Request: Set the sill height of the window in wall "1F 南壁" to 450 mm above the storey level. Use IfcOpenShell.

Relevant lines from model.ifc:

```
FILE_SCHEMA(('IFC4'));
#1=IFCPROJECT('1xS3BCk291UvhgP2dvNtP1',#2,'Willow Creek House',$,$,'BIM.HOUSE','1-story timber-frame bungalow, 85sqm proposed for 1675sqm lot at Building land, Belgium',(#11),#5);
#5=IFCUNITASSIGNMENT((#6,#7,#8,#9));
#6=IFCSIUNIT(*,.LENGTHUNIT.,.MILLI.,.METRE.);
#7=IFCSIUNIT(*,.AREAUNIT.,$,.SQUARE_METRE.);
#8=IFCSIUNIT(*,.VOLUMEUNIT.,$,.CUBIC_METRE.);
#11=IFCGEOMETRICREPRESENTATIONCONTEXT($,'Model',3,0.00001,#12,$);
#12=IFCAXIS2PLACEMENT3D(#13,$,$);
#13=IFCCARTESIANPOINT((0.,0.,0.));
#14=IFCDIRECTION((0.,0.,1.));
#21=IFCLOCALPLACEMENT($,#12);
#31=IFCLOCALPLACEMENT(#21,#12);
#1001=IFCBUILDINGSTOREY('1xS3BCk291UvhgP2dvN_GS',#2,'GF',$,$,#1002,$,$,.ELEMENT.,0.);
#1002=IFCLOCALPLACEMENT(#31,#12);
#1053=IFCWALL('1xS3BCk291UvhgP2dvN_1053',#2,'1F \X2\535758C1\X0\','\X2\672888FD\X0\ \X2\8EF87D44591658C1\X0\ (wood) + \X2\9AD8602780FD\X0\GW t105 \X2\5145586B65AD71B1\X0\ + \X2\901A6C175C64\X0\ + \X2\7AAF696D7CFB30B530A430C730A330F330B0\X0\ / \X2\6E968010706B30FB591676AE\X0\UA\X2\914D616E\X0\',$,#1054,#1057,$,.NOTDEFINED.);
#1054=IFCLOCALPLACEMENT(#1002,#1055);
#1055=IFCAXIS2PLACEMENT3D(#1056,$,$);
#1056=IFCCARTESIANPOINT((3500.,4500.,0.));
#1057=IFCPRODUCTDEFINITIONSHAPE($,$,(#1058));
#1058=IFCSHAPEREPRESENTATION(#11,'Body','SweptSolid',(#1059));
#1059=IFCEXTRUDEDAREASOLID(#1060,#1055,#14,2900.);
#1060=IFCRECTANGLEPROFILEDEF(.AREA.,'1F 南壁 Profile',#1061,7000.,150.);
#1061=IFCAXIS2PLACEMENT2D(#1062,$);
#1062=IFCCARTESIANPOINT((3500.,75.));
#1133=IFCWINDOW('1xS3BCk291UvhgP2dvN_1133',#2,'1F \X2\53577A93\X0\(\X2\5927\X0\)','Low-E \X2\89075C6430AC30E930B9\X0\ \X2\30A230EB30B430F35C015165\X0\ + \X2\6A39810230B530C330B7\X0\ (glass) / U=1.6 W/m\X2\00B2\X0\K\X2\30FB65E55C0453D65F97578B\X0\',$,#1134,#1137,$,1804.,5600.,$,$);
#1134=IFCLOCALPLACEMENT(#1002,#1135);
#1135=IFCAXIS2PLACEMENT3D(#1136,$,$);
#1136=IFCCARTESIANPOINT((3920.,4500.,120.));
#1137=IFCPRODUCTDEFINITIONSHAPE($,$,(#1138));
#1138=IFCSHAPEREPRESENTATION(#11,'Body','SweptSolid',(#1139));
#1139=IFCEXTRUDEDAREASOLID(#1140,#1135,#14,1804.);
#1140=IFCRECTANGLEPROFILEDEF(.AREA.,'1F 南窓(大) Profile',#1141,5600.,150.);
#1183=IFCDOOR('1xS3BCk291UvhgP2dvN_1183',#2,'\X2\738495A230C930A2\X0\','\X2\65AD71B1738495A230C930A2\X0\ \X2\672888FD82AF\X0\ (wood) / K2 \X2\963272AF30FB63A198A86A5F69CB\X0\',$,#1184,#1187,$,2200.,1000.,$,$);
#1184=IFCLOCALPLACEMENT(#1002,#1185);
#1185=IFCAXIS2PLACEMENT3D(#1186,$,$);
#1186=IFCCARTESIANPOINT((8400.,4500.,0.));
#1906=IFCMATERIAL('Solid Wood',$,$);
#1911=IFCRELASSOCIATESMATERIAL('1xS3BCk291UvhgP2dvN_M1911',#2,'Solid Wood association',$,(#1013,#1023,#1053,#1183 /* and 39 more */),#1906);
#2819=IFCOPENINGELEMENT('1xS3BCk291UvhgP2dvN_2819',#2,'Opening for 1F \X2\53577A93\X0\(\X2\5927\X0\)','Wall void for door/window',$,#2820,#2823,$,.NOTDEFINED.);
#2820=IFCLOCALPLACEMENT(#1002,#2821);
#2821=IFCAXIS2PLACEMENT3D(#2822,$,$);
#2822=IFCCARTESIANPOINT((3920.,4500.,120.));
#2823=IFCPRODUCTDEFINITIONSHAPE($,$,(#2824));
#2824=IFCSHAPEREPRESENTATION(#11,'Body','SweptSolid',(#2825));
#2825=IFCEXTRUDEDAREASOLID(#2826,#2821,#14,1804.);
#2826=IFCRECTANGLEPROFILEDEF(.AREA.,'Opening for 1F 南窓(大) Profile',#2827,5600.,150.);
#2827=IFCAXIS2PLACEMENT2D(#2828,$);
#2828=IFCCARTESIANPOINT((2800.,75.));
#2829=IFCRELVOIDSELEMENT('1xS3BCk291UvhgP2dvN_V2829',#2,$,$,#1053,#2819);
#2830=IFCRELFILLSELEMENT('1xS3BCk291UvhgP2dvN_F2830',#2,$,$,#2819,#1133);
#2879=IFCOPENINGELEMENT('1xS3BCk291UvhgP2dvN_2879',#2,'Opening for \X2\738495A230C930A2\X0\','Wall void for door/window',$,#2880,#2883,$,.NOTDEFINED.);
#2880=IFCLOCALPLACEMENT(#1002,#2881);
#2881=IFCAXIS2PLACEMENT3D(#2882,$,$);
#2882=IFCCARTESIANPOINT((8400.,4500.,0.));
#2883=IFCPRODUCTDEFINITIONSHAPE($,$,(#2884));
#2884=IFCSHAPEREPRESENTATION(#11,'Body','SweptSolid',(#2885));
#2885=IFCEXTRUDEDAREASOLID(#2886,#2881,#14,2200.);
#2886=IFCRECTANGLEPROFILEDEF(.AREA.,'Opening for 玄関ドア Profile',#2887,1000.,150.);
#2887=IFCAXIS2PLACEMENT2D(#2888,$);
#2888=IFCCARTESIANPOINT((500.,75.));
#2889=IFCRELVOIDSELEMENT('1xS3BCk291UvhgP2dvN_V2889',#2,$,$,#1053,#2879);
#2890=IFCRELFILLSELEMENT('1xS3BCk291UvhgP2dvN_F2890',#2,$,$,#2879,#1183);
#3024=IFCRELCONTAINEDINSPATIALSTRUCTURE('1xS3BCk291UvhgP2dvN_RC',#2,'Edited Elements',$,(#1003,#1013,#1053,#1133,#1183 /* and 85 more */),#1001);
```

```python
import numpy as np
import ifcopenshell
import ifcopenshell.api.geometry
import ifcopenshell.geom
import ifcopenshell.util.element
import ifcopenshell.util.placement
import ifcopenshell.util.shape
import ifcopenshell.util.unit

model = ifcopenshell.open("model.ifc")
unit_scale = ifcopenshell.util.unit.calculate_unit_scale(model)

window = model.by_guid("1xS3BCk291UvhgP2dvN_1133")
opening = window.FillsVoids[0].RelatingOpeningElement
storey = ifcopenshell.util.element.get_container(window, ifc_class="IfcBuildingStorey")
level = ifcopenshell.util.placement.get_local_placement(storey.ObjectPlacement)[2, 3]

# The opening's origin need not be at the sill, so measure its lowest point.
shape = ifcopenshell.geom.create_shape(ifcopenshell.geom.settings(), opening)
bottom = ifcopenshell.util.shape.get_shape_bottom_elevation(shape, shape.geometry) / unit_scale
dz = level + 450.0 - bottom

shift = np.array([0.0, 0.0, dz])
# The window is not placed relative to its opening, so move both.
for product in (opening, window):
    matrix = ifcopenshell.util.placement.get_local_placement(product.ObjectPlacement)
    matrix[:3, 3] += shift
    ifcopenshell.api.geometry.edit_object_placement(model, product=product, matrix=matrix, is_si=False)

print(f"moved by {dz * unit_scale:+.3f} m")

model.write("model-out.ifc")
```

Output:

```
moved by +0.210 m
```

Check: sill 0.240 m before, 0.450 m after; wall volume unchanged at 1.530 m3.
